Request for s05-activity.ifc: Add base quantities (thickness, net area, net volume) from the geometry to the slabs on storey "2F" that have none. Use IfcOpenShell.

First a look at what the model holds.

```python
import ifcopenshell
import ifcopenshell.util.element
import ifcopenshell.util.unit

model = ifcopenshell.open("s05-activity.ifc")
print(model.schema)
for unit_type in ("LENGTHUNIT", "AREAUNIT", "VOLUMEUNIT"):
    print(unit_type, ifcopenshell.util.unit.calculate_unit_scale(model, unit_type))
storey = next(s for s in model.by_type("IfcBuildingStorey") if s.Name == "2F")
slabs = [e for e in ifcopenshell.util.element.get_decomposition(storey) if e.is_a("IfcSlab")]
for e in sorted(slabs, key=lambda e: e.id()):
    print(e.id(), e.is_a(), e.Name, list(ifcopenshell.util.element.get_psets(e, qtos_only=True)), sep=" | ")
```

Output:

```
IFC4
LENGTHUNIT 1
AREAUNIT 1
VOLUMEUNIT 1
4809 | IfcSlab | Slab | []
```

```python
import ifcopenshell
import ifcopenshell.api.pset
import ifcopenshell.geom
import ifcopenshell.util.element
import ifcopenshell.util.shape
import ifcopenshell.util.unit

model = ifcopenshell.open("s05-activity.ifc")
unit_scale = ifcopenshell.util.unit.calculate_unit_scale(model)
area_scale = ifcopenshell.util.unit.calculate_unit_scale(model, "AREAUNIT")
volume_scale = ifcopenshell.util.unit.calculate_unit_scale(model, "VOLUMEUNIT")
settings = ifcopenshell.geom.settings()

storey = next(s for s in model.by_type("IfcBuildingStorey") if s.Name == "2F")
slabs = [e for e in ifcopenshell.util.element.get_decomposition(storey) if e.is_a("IfcSlab")]

for e in sorted(slabs, key=lambda e: e.id()):
    if ifcopenshell.util.element.get_psets(e, qtos_only=True, should_inherit=False):
        continue
    # Geometry comes back in metres, in the element's own axes.
    shape = ifcopenshell.geom.create_shape(settings, e)
    values = {
        "Width": ifcopenshell.util.shape.get_z(shape.geometry) / unit_scale,
        "NetArea": ifcopenshell.util.shape.get_footprint_area(shape.geometry) / area_scale,
        "NetVolume": ifcopenshell.util.shape.get_volume(shape.geometry) / volume_scale,
    }
    qto = ifcopenshell.api.pset.add_qto(model, product=e, name="Qto_SlabBaseQuantities")
    ifcopenshell.api.pset.edit_qto(model, qto=qto, properties=values)
    print(e.id(), {k: round(v, 3) for k, v in values.items()})

model.write("s05-activity-out.ifc")
```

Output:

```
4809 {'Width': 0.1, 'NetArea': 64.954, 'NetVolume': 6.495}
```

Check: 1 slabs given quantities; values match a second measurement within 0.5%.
